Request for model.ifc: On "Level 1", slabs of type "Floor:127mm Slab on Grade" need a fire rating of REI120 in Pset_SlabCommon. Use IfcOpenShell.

First a look at what the model holds.

```python
import ifcopenshell
import ifcopenshell.util.element

model = ifcopenshell.open("model.ifc")
print(model.schema)
storey = next(s for s in model.by_type("IfcBuildingStorey") if s.Name == "Level 1")
slabs = [e for e in ifcopenshell.util.element.get_decomposition(storey) if e.is_a("IfcSlab")]
seen = {}
for e in slabs:
    element_type = ifcopenshell.util.element.get_type(e)
    key = (element_type.Name if element_type != e and element_type else None, ifcopenshell.util.element.get_pset(e, "Pset_SlabCommon", "FireRating"))
    seen[key] = seen.get(key, 0) + 1
for (name, value), count in sorted(seen.items(), key=str):
    print(count, "x", name, "|", value)
```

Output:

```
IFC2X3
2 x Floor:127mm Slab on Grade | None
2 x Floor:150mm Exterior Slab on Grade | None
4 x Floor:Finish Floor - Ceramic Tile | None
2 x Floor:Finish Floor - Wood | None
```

```python
import ifcopenshell
import ifcopenshell.api.pset
import ifcopenshell.util.element

model = ifcopenshell.open("model.ifc")

storey = next(s for s in model.by_type("IfcBuildingStorey") if s.Name == "Level 1")
slabs = [e for e in ifcopenshell.util.element.get_decomposition(storey) if e.is_a("IfcSlab")]

count = 0
for e in slabs:
    element_type = ifcopenshell.util.element.get_type(e)
    if element_type in (None, e) or element_type.Name != "Floor:127mm Slab on Grade":
        continue
    # add_pset returns the element's existing set when there is one.
    pset = ifcopenshell.api.pset.add_pset(model, product=e, name="Pset_SlabCommon")
    ifcopenshell.api.pset.edit_pset(model, pset=pset, properties={"FireRating": "REI120"})
    count += 1

print(count, "slabs updated")

model.write("model_v2.ifc")
```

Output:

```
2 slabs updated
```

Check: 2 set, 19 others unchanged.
